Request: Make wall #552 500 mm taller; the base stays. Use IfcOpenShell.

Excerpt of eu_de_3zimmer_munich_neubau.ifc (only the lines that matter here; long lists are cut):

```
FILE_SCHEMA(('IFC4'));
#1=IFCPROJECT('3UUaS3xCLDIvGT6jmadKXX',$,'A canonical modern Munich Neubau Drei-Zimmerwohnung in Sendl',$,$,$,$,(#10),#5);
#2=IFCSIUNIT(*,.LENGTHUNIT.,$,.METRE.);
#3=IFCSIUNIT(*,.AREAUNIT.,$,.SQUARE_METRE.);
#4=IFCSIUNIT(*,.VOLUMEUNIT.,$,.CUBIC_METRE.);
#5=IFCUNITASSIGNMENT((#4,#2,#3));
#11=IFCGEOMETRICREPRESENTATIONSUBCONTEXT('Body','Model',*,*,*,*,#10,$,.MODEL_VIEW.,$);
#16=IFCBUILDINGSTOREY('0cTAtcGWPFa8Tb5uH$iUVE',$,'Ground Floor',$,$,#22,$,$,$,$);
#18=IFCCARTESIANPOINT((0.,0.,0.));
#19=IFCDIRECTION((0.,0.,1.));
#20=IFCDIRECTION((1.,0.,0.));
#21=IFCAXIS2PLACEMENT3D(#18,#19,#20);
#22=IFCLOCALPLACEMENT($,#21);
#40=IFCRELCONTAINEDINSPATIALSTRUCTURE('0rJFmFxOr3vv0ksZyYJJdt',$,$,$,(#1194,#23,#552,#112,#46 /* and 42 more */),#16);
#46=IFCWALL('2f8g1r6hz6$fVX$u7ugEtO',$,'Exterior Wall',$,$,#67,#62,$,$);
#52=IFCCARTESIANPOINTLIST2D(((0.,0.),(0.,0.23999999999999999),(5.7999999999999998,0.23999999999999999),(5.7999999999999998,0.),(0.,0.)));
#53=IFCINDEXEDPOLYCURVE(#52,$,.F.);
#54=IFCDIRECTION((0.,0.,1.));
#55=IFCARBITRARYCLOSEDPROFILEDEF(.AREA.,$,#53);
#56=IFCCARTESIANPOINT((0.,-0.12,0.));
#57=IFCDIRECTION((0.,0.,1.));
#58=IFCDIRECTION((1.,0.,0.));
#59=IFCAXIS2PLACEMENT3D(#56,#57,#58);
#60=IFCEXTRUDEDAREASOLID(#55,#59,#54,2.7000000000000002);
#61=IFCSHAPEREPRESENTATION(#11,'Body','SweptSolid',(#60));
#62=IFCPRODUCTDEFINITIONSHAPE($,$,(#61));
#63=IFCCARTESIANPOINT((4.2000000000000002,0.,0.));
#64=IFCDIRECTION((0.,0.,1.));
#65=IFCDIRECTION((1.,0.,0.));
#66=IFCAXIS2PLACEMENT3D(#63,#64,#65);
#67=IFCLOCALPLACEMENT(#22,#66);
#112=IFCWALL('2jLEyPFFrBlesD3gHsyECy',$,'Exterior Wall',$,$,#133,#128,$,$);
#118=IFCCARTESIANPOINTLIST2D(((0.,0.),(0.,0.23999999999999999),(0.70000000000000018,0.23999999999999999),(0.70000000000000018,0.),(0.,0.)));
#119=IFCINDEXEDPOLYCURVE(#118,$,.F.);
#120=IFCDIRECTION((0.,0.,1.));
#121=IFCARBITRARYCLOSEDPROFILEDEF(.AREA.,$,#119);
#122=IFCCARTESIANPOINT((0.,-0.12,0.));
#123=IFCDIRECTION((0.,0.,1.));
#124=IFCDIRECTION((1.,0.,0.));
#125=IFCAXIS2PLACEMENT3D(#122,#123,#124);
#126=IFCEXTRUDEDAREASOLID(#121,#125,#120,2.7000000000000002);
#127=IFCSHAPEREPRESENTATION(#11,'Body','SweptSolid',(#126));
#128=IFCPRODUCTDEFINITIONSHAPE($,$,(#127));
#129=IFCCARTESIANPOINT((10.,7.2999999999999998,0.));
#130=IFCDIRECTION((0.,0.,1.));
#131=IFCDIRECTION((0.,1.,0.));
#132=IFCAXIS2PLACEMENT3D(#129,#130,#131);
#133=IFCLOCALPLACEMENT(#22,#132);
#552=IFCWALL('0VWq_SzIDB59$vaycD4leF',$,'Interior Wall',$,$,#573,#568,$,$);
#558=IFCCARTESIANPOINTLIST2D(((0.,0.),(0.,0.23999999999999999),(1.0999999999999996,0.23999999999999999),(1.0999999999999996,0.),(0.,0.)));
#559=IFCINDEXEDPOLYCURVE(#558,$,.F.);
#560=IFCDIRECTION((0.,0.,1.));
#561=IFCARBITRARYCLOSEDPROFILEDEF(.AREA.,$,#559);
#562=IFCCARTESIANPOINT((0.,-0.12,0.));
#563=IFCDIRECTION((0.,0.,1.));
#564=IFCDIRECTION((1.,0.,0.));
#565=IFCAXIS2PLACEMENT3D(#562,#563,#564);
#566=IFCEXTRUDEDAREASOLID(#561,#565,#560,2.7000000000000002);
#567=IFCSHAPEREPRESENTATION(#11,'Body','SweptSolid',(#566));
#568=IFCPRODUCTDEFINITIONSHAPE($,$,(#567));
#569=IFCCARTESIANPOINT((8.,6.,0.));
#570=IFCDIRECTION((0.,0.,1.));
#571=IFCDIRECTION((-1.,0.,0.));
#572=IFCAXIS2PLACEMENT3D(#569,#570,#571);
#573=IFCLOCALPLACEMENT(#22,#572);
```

```python
import ifcopenshell
import ifcopenshell.geom
import ifcopenshell.util.representation
import ifcopenshell.util.shape

model = ifcopenshell.open("eu_de_3zimmer_munich_neubau.ifc")
settings = ifcopenshell.geom.settings()


def volume(element):
    """Net volume in cubic metres, openings subtracted."""
    shape = ifcopenshell.geom.create_shape(settings, element)
    return ifcopenshell.util.shape.get_volume(shape.geometry)


wall = model.by_id(552)
before = volume(wall)

body = ifcopenshell.util.representation.get_representation(wall, "Model", "Body")
solid = body.Items[0]
old_height = solid.Depth
solid.Depth += 0.5
after = volume(wall)

print(f"height {old_height:g} -> {solid.Depth:g}, volume {before:.3f} -> {after:.3f} m3")

model.write("eu_de_3zimmer_munich_neubau_rev.ifc")
```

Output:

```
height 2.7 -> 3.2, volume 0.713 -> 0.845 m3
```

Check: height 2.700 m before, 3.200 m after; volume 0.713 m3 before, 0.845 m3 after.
